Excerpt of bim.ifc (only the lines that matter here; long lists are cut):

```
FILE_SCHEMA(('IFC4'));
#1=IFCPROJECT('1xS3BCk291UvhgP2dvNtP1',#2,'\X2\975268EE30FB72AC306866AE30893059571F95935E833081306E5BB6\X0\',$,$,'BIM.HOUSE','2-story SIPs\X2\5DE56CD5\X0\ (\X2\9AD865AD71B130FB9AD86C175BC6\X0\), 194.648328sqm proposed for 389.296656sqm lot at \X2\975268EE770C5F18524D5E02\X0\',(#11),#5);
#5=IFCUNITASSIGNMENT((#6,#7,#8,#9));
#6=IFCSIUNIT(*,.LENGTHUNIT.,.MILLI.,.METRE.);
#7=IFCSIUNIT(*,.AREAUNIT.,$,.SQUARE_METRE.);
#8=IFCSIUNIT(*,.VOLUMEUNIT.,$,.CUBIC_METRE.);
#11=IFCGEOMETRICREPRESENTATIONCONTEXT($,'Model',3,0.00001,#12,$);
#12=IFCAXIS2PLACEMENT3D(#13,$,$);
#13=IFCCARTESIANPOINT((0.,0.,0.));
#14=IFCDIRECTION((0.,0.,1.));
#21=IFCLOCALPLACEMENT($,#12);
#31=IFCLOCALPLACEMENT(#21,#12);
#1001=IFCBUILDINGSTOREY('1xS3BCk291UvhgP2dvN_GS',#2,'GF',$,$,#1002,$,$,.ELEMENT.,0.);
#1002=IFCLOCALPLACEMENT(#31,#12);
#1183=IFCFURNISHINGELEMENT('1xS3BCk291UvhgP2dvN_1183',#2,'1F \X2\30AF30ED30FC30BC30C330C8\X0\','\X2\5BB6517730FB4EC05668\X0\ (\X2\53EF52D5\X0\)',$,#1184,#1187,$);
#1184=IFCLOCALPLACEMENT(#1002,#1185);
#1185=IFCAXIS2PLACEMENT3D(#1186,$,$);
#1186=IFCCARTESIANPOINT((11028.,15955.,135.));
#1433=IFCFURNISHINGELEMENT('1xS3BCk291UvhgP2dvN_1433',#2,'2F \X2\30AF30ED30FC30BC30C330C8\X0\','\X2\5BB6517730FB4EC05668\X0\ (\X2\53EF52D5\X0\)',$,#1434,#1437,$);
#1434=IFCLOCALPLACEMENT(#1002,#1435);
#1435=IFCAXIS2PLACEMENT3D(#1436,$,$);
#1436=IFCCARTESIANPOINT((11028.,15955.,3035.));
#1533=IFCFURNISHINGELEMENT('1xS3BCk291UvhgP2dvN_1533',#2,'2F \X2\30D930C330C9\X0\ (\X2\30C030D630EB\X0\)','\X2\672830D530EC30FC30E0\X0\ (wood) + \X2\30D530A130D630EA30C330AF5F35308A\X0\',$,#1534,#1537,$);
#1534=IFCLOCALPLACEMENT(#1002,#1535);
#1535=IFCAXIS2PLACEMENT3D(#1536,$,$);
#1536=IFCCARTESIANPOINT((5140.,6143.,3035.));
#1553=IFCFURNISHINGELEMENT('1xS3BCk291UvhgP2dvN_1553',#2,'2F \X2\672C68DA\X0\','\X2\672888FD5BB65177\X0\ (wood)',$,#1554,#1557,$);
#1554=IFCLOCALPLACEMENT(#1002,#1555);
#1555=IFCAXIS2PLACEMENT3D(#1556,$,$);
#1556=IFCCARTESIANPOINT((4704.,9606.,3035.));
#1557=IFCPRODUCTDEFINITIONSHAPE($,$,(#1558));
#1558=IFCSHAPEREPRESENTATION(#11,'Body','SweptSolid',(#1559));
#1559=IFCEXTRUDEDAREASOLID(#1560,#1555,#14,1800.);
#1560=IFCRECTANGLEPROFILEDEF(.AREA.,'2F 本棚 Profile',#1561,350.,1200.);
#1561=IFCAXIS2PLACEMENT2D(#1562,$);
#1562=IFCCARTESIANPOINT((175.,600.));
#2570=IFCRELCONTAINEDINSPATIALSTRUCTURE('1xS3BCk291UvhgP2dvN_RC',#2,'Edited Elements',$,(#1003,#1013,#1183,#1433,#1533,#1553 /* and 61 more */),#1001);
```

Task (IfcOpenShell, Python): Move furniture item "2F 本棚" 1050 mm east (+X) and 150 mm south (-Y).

```python
import ifcopenshell
import ifcopenshell.api.geometry
import ifcopenshell.util.placement
import ifcopenshell.util.unit

model = ifcopenshell.open("bim.ifc")
unit_scale = ifcopenshell.util.unit.calculate_unit_scale(model)

item = model.by_guid("1xS3BCk291UvhgP2dvN_1553")
matrix = ifcopenshell.util.placement.get_local_placement(item.ObjectPlacement)
matrix[0, 3] += 1.05 / unit_scale
matrix[1, 3] -= 0.15 / unit_scale
ifcopenshell.api.geometry.edit_object_placement(model, product=item, matrix=matrix, is_si=False)

print(ifcopenshell.util.placement.get_local_placement(item.ObjectPlacement).round(3) + 0.0)

model.write("bim-out.ifc")
```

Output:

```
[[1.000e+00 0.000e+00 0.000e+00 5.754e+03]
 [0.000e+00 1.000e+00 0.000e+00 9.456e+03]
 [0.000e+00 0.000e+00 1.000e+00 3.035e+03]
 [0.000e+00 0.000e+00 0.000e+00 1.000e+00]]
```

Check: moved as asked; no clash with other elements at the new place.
